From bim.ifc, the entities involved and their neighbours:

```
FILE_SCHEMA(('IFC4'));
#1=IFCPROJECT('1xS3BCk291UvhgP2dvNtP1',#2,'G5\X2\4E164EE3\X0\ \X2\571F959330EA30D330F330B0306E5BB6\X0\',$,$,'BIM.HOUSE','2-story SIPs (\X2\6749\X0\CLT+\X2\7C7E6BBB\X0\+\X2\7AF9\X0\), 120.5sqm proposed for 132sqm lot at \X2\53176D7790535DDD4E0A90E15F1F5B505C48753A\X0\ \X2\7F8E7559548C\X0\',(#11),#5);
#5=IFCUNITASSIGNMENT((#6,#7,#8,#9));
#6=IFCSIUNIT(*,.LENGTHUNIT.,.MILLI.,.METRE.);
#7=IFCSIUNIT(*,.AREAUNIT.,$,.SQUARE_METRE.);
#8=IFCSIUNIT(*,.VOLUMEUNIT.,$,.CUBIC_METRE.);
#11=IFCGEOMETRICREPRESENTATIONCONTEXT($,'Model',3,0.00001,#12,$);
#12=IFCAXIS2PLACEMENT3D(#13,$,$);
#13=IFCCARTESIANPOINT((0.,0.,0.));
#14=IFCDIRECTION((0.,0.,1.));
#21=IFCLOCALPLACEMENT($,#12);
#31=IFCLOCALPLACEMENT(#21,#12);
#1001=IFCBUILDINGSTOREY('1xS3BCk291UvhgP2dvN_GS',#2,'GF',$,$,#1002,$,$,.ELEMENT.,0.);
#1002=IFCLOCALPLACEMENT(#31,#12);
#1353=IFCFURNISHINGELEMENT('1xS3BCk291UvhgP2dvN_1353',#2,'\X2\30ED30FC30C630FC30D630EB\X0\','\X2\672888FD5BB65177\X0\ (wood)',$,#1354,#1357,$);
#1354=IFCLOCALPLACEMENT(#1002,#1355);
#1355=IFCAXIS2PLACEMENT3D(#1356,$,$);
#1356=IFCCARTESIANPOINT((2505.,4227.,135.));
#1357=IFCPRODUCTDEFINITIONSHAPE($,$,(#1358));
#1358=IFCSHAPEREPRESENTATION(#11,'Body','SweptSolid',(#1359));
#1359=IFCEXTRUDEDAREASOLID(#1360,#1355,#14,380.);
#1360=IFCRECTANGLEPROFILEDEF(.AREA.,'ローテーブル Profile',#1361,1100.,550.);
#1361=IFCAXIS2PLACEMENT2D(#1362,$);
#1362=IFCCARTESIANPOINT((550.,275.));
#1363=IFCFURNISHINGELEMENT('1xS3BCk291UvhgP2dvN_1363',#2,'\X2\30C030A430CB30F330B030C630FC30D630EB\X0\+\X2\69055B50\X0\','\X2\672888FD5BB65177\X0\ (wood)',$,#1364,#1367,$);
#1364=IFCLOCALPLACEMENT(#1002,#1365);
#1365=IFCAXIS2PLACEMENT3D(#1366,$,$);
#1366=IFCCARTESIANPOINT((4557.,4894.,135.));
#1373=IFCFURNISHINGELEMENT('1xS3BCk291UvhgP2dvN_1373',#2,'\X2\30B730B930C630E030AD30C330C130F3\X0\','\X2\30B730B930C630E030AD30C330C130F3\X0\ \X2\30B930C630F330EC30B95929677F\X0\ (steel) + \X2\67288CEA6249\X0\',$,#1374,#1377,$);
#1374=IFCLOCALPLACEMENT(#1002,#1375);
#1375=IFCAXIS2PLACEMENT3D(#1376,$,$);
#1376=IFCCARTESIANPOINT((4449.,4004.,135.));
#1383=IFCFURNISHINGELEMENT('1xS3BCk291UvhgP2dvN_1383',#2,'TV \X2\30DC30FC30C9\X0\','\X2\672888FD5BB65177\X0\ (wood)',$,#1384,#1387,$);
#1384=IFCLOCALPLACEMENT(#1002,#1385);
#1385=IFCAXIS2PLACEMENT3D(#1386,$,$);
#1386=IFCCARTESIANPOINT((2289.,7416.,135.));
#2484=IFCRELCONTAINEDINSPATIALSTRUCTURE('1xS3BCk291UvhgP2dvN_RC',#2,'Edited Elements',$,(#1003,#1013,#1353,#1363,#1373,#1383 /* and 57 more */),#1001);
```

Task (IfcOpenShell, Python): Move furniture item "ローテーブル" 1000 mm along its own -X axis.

```python
import ifcopenshell
import ifcopenshell.api.geometry
import ifcopenshell.util.placement
import ifcopenshell.util.unit

model = ifcopenshell.open("bim.ifc")
unit_scale = ifcopenshell.util.unit.calculate_unit_scale(model)

item = model.by_guid("1xS3BCk291UvhgP2dvN_1353")
matrix = ifcopenshell.util.placement.get_local_placement(item.ObjectPlacement)
matrix[:3, 3] -= matrix[:3, 0] * 1 / unit_scale
ifcopenshell.api.geometry.edit_object_placement(model, product=item, matrix=matrix, is_si=False)

print(ifcopenshell.util.placement.get_local_placement(item.ObjectPlacement).round(3) + 0.0)

model.write("bim_edited.ifc")
```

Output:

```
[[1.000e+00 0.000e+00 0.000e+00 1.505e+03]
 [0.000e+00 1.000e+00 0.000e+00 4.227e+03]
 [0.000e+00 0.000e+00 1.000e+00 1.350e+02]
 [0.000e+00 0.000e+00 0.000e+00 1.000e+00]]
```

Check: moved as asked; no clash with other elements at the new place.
